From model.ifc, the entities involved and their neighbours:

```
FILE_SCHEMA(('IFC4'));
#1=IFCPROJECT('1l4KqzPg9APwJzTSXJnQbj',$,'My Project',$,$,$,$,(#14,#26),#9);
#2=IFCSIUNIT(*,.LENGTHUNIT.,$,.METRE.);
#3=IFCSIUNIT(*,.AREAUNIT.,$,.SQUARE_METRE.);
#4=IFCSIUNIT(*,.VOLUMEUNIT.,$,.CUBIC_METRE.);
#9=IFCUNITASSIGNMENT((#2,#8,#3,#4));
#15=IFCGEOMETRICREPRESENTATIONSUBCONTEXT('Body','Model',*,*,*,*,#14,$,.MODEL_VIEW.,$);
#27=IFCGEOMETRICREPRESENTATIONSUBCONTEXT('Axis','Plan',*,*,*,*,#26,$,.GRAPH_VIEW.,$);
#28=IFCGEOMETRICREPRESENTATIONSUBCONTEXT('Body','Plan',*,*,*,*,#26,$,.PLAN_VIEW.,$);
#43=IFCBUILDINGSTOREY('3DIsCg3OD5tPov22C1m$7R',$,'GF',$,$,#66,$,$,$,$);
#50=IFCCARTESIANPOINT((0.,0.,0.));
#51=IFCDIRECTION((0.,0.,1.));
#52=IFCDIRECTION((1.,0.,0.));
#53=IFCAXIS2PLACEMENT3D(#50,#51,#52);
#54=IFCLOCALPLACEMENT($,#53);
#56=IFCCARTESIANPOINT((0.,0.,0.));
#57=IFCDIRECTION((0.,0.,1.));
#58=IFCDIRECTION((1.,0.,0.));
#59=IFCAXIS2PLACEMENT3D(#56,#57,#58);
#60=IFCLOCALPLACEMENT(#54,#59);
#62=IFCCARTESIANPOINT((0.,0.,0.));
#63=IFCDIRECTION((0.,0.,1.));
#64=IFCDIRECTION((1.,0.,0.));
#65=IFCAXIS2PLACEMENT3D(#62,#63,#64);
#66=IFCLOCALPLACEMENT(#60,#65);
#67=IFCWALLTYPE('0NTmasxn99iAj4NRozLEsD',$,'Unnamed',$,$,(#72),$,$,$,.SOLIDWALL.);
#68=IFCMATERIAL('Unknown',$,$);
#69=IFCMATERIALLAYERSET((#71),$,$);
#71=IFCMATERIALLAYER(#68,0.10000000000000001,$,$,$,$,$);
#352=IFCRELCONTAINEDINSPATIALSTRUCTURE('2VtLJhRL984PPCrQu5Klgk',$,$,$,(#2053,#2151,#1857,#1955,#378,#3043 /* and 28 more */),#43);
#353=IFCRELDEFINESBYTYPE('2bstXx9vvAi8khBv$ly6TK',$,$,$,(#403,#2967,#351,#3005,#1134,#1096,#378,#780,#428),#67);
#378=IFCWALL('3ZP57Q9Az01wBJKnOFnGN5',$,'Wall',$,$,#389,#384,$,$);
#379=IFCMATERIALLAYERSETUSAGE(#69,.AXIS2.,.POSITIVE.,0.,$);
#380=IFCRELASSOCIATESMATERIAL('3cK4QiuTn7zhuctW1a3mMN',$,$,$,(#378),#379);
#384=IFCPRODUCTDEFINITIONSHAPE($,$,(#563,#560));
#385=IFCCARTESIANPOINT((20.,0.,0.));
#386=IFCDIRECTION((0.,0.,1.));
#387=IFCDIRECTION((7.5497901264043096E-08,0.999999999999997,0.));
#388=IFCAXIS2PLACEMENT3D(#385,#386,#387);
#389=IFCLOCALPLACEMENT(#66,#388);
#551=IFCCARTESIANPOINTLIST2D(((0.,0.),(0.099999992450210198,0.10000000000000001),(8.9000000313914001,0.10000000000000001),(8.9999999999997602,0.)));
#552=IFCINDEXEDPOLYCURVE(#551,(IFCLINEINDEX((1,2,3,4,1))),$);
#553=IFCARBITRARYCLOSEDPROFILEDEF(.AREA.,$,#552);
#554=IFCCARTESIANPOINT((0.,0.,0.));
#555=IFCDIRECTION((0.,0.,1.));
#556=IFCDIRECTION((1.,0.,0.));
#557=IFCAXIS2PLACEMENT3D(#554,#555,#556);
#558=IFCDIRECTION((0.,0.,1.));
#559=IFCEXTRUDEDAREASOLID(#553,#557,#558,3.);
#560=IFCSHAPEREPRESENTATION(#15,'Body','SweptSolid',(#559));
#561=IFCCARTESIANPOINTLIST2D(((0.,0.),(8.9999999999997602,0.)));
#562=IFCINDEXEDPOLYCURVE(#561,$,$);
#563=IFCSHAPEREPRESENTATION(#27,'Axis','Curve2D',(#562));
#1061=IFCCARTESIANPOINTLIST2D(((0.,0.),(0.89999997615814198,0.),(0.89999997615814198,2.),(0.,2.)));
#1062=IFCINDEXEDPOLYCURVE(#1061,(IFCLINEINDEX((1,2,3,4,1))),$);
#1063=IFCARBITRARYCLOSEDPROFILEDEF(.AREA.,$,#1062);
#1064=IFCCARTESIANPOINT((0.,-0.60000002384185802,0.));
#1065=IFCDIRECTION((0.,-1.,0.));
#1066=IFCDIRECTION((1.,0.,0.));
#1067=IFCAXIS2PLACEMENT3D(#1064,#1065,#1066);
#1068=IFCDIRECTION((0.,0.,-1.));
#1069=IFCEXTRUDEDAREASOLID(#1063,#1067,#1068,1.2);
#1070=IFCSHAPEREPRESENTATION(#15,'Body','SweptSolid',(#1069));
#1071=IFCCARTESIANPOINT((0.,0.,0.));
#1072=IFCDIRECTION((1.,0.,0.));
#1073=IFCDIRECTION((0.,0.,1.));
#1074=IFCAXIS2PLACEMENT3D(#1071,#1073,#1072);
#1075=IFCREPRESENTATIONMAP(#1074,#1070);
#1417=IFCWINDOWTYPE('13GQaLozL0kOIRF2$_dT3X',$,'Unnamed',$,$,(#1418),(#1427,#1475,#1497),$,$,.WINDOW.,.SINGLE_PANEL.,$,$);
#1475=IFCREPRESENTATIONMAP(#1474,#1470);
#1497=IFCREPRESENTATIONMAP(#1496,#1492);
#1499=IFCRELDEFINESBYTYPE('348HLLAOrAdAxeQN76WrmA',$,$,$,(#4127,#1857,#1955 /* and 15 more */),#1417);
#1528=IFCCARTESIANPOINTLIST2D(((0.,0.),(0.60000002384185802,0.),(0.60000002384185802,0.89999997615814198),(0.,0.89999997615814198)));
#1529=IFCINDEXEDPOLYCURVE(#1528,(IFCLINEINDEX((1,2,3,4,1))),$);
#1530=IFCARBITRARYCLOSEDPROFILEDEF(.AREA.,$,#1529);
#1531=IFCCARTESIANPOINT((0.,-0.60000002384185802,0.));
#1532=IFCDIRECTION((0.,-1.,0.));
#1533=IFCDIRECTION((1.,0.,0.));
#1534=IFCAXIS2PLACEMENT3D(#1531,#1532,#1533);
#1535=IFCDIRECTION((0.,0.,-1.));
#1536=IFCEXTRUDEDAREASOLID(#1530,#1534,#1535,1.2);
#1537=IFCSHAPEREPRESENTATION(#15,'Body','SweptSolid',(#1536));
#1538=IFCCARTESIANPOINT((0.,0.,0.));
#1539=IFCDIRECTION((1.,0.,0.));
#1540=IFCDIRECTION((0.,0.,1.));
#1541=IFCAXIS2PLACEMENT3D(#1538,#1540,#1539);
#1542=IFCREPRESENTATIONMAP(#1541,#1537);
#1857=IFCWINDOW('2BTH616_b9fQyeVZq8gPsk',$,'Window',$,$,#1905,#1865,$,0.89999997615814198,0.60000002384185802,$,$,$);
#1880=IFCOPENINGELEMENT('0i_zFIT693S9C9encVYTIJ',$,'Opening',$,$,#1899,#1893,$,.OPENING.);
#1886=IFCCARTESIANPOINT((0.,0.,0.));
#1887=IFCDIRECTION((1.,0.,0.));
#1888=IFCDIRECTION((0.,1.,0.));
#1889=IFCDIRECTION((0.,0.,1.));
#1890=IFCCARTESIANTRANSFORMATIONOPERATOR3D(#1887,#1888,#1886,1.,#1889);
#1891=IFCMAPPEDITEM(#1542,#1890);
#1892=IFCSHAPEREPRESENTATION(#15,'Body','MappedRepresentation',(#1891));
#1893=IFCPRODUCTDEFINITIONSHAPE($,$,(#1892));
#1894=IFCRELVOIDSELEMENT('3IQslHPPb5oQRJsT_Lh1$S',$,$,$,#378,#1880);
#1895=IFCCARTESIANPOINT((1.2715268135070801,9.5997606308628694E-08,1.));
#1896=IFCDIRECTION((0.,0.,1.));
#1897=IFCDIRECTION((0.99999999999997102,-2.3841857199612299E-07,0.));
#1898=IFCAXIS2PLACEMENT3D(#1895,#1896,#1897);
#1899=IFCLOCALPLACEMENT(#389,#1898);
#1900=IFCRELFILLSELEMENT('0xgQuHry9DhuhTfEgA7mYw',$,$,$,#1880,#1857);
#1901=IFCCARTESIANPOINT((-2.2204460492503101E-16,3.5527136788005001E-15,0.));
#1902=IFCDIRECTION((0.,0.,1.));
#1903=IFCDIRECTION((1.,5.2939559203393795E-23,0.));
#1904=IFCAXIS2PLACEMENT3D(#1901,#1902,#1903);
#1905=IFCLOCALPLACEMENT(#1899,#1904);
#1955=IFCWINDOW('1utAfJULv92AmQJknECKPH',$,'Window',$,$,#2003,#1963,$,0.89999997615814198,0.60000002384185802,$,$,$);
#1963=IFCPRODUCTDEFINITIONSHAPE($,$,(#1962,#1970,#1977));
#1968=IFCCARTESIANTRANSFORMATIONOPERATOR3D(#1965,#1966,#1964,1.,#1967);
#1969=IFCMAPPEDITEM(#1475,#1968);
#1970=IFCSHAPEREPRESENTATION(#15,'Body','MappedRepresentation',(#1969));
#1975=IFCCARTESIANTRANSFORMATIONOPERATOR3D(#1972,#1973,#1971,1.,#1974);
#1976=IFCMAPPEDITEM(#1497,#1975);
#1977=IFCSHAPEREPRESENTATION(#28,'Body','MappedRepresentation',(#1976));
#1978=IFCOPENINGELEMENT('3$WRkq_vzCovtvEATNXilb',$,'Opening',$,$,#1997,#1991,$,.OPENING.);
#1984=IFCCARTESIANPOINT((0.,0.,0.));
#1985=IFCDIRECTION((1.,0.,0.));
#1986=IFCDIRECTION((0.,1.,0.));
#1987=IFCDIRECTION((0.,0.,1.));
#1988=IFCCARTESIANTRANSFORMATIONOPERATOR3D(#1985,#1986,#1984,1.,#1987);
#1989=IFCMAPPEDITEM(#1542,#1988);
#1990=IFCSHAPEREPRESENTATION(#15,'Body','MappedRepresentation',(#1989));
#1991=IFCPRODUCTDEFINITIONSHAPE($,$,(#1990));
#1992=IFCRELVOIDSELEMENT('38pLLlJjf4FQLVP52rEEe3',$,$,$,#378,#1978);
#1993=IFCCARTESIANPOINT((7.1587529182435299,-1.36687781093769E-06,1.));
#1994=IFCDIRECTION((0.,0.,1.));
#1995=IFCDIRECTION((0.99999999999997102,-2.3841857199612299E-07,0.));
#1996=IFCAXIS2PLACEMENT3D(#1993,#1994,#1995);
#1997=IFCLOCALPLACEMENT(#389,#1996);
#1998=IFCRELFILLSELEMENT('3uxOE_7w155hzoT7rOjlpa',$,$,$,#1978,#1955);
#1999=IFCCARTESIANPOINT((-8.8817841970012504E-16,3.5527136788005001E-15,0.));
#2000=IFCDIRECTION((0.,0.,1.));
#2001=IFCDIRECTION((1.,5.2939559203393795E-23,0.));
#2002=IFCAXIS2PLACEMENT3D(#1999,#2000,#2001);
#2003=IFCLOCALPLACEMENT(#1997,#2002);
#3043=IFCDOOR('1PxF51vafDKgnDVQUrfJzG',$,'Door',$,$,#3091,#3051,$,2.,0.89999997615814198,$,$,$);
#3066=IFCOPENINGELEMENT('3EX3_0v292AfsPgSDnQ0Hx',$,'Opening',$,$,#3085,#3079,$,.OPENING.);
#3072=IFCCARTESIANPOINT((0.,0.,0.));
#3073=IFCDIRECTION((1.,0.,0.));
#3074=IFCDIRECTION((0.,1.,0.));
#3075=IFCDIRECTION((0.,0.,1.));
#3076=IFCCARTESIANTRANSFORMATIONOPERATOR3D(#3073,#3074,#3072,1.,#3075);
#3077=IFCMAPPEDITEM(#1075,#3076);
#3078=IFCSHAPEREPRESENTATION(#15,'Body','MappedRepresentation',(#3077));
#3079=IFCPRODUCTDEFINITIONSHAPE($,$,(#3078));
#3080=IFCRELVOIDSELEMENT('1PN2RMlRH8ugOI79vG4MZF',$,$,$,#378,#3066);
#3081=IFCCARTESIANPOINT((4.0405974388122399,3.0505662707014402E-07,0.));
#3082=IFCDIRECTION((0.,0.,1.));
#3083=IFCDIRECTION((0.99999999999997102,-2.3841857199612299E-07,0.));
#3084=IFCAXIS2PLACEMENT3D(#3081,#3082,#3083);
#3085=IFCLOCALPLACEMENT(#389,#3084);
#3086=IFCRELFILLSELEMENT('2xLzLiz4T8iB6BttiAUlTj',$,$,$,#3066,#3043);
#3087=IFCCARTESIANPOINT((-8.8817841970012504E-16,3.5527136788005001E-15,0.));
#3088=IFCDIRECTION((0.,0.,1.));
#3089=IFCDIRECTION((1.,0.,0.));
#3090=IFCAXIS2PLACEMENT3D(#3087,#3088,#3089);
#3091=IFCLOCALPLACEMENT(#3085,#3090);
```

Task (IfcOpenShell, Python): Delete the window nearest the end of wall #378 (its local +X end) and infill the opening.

```python
import ifcopenshell
import ifcopenshell.api.feature
import ifcopenshell.api.root
import ifcopenshell.geom
import ifcopenshell.util.shape

model = ifcopenshell.open("model.ifc")
settings = ifcopenshell.geom.settings()


def volume(element):
    """Net volume in cubic metres, openings subtracted."""
    shape = ifcopenshell.geom.create_shape(settings, element)
    return ifcopenshell.util.shape.get_volume(shape.geometry)


window = model.by_guid("1utAfJULv92AmQJknECKPH")
opening = window.FillsVoids[0].RelatingOpeningElement
wall = opening.VoidsElements[0].RelatingBuildingElement
before = volume(wall)

ifcopenshell.api.root.remove_product(model, product=window)
ifcopenshell.api.feature.remove_feature(model, feature=opening)

after = volume(wall)

print(f"wall volume {before:.3f} -> {after:.3f} m3")

model.write("model_rev.ifc")
```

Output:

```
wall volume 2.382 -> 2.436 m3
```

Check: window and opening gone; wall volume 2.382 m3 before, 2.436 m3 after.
